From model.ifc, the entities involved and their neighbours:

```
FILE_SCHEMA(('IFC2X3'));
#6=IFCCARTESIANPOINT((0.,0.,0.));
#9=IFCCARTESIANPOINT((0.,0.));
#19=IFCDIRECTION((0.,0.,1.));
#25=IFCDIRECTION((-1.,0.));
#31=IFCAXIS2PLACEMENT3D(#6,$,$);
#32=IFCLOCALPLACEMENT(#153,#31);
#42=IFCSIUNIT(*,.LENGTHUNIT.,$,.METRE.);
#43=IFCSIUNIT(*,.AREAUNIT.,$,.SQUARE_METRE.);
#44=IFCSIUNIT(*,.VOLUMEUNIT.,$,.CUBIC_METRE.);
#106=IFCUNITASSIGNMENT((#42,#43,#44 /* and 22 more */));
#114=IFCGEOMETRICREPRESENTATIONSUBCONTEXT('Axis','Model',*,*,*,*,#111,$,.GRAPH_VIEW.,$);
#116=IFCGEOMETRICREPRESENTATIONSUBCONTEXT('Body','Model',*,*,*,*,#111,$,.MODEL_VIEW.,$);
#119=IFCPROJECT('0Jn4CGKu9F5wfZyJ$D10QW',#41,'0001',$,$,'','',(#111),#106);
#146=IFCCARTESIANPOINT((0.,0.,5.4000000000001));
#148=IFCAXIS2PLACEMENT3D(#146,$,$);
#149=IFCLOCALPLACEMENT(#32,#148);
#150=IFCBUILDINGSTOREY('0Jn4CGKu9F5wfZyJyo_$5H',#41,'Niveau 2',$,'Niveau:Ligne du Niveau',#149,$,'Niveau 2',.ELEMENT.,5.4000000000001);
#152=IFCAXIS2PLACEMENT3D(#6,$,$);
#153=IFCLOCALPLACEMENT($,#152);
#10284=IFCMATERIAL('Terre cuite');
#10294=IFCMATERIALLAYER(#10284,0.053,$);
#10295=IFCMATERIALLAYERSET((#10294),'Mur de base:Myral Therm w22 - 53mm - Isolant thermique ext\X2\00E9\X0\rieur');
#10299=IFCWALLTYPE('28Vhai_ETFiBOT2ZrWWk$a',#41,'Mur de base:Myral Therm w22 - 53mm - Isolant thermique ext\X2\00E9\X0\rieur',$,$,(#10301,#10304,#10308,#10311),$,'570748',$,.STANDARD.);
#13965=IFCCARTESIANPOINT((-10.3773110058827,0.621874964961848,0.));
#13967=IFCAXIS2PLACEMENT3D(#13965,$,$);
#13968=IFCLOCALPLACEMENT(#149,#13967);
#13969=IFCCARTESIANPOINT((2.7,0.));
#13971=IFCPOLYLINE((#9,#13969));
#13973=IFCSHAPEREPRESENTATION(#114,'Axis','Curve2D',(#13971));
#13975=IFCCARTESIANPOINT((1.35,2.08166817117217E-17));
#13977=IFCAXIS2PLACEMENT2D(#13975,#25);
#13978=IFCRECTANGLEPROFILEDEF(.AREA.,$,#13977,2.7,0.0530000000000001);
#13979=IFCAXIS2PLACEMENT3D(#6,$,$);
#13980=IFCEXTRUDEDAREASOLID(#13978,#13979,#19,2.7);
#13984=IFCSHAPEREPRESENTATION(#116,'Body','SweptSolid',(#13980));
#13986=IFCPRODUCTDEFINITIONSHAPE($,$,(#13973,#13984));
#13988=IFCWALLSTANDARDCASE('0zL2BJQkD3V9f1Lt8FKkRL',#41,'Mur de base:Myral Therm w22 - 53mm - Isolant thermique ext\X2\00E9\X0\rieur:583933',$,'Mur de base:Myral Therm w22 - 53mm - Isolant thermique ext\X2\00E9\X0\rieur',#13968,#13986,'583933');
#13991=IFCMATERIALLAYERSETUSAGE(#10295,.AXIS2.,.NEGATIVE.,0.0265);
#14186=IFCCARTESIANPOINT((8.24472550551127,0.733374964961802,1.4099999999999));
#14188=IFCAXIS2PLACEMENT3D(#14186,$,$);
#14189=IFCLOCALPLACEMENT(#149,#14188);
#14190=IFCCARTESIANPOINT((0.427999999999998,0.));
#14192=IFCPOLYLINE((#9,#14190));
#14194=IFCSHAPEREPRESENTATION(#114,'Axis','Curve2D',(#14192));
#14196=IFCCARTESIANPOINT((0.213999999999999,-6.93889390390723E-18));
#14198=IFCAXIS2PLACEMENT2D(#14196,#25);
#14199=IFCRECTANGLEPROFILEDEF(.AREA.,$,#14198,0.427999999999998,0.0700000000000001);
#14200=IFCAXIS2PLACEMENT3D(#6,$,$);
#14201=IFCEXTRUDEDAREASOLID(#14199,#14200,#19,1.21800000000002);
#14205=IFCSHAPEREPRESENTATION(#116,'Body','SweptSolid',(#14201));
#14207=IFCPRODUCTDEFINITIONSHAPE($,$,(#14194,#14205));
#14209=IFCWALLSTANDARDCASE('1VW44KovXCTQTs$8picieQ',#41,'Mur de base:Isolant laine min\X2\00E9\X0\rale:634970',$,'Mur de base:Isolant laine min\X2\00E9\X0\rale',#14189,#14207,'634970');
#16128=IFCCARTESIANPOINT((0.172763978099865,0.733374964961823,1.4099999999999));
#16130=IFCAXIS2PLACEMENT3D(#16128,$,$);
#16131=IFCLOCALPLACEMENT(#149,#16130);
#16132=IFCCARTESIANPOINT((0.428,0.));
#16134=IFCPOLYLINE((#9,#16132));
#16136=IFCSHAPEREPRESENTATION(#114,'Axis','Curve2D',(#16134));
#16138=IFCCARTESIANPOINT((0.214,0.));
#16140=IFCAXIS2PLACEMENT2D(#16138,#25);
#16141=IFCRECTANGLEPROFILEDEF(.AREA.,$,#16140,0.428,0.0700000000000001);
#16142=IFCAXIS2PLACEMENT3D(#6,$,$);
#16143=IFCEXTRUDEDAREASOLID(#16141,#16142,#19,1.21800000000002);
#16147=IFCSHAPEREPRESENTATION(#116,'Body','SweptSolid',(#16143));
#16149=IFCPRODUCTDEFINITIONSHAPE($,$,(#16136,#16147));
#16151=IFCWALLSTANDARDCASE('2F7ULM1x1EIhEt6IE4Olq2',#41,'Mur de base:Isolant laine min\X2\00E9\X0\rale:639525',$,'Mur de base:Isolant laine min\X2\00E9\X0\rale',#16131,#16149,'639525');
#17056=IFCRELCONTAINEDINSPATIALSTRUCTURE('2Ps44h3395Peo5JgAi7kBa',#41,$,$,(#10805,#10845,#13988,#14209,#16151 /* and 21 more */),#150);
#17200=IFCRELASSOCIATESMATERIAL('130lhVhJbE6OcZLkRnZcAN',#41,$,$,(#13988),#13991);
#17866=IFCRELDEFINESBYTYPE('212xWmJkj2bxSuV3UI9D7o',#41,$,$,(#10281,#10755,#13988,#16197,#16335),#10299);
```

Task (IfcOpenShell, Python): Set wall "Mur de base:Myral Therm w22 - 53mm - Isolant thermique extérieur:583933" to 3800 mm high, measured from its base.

```python
import ifcopenshell
import ifcopenshell.geom
import ifcopenshell.util.representation
import ifcopenshell.util.shape

model = ifcopenshell.open("model.ifc")
settings = ifcopenshell.geom.settings()


def volume(element):
    """Net volume in cubic metres, openings subtracted."""
    shape = ifcopenshell.geom.create_shape(settings, element)
    return ifcopenshell.util.shape.get_volume(shape.geometry)


wall = model.by_id(13988)
before = volume(wall)

body = ifcopenshell.util.representation.get_representation(wall, "Model", "Body")
solid = body.Items[0]
old_height = solid.Depth
solid.Depth = 3.8
after = volume(wall)

print(f"height {old_height:g} -> {solid.Depth:g}, volume {before:.3f} -> {after:.3f} m3")

model.write("model_rev.ifc")
```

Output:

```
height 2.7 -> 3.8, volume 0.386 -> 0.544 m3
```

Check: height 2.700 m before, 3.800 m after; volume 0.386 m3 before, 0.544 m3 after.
